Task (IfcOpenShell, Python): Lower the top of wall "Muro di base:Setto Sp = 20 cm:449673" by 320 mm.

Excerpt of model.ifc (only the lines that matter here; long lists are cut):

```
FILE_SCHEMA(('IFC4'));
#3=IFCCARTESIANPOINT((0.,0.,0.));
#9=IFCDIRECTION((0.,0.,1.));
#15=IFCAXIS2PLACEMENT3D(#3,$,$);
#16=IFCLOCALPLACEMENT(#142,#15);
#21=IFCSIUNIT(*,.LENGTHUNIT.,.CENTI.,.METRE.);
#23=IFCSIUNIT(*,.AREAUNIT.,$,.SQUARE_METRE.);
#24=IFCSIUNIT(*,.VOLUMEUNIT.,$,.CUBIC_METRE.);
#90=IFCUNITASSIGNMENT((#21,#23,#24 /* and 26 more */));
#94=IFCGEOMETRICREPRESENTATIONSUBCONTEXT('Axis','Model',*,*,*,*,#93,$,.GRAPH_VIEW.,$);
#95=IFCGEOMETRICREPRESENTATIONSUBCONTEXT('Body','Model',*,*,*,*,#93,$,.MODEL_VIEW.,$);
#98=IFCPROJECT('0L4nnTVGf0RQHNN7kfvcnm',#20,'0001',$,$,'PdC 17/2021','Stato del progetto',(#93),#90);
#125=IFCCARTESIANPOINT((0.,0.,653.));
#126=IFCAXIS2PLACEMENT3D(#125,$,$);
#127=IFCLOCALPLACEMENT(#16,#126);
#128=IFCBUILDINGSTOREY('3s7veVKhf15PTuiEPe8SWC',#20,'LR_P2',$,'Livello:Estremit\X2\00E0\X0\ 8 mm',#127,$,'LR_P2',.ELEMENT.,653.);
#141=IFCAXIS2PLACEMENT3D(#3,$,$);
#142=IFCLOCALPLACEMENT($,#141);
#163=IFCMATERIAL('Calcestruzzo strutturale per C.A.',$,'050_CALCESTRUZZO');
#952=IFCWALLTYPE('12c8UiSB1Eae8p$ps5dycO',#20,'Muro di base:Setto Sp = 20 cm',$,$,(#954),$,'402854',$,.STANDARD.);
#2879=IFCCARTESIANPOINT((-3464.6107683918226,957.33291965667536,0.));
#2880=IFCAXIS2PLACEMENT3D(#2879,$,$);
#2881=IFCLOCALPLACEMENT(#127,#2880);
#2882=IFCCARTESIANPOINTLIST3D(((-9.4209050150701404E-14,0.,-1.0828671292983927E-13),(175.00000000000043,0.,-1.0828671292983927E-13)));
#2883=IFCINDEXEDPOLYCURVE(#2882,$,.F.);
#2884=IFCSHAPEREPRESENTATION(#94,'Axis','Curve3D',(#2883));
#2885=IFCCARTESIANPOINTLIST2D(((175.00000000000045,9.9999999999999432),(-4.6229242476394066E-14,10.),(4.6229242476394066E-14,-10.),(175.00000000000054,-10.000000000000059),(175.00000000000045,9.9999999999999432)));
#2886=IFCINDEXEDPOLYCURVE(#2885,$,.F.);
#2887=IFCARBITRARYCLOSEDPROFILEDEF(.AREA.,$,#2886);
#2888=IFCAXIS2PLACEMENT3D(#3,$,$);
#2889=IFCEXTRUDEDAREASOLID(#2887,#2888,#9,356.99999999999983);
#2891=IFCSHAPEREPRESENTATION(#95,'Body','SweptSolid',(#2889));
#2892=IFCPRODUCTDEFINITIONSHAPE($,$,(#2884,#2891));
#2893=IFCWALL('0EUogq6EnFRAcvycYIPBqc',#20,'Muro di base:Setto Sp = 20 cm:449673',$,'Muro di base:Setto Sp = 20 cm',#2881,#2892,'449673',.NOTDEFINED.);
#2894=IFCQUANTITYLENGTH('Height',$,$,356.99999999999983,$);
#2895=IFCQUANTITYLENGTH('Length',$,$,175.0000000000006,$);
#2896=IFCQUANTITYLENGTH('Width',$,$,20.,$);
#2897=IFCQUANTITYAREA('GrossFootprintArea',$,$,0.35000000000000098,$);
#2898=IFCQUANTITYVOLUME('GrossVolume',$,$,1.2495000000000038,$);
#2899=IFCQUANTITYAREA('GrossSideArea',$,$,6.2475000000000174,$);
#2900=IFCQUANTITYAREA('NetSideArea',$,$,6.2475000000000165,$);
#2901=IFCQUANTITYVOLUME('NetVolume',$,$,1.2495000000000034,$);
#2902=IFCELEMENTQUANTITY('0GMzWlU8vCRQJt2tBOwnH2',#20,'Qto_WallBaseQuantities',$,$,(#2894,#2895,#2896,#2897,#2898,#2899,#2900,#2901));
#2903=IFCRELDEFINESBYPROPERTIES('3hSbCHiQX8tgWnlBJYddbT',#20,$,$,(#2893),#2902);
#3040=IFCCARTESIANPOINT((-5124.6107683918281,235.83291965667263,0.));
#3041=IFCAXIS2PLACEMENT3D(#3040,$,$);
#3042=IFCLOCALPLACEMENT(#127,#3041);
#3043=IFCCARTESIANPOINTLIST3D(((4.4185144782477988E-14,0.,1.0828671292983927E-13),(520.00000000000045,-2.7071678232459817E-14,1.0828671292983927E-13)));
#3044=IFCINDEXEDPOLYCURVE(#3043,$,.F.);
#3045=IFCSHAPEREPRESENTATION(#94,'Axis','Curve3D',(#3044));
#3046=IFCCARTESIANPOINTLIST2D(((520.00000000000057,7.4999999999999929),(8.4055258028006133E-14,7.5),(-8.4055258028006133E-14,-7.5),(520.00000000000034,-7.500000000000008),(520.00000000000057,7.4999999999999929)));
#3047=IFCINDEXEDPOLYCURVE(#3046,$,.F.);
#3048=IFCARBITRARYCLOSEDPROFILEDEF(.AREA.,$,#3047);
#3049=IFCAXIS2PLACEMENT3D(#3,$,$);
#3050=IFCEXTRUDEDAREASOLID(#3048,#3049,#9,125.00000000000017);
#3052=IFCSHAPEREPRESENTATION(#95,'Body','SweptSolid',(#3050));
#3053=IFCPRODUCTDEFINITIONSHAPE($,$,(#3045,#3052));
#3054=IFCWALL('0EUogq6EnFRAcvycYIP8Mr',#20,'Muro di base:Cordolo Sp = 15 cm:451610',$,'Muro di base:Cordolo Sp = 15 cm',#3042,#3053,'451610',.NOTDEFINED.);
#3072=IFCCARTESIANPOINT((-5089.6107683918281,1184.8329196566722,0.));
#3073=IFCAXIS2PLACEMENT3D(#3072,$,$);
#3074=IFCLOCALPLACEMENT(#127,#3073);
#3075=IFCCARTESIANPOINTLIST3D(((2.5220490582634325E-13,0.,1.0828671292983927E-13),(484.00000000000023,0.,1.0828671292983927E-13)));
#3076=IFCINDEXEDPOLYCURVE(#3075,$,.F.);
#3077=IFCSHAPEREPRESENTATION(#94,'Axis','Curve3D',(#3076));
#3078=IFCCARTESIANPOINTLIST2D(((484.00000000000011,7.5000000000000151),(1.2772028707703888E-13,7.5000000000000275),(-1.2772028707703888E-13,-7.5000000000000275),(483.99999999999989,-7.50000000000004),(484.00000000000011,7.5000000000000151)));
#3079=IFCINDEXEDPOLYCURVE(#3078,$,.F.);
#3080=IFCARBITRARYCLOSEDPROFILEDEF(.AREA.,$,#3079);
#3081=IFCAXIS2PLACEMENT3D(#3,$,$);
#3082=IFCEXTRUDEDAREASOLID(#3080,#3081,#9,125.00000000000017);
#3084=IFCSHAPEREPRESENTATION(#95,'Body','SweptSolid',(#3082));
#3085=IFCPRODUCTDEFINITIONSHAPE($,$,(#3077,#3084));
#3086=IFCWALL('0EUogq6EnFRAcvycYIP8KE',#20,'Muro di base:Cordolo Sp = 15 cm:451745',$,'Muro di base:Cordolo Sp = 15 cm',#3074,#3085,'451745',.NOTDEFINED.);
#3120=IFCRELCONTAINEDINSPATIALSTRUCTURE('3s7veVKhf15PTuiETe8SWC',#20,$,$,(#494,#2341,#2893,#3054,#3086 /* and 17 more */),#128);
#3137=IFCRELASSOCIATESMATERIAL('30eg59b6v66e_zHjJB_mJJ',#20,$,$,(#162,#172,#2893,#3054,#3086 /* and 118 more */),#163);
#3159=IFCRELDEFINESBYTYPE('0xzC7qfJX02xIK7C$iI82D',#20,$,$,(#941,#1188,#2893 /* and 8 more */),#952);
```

```python
import ifcopenshell
import ifcopenshell.api.pset
import ifcopenshell.geom
import ifcopenshell.util.element
import ifcopenshell.util.representation
import ifcopenshell.util.shape
import ifcopenshell.util.unit

model = ifcopenshell.open("model.ifc")
unit_scale = ifcopenshell.util.unit.calculate_unit_scale(model)
area_scale = ifcopenshell.util.unit.calculate_unit_scale(model, "AREAUNIT")
volume_scale = ifcopenshell.util.unit.calculate_unit_scale(model, "VOLUMEUNIT")
settings = ifcopenshell.geom.settings()


def volume(element):
    """Net volume in cubic metres, openings subtracted."""
    shape = ifcopenshell.geom.create_shape(settings, element)
    return ifcopenshell.util.shape.get_volume(shape.geometry)


wall = model.by_guid("0EUogq6EnFRAcvycYIPBqc")
before = volume(wall)

body = ifcopenshell.util.representation.get_representation(wall, "Model", "Body")
solid = body.Items[0]
old_height = solid.Depth
solid.Depth -= 0.32 / unit_scale
after = volume(wall)
thickness = 0.2  # wall thickness in metres

# Update the stored height, areas and volumes.
qto = model.by_id(ifcopenshell.util.element.get_pset(wall, "Qto_WallBaseQuantities", should_inherit=False)["id"])
ifcopenshell.api.pset.edit_qto(model, qto=qto, properties={
    "Height": solid.Depth,
    "GrossVolume": ifcopenshell.util.element.get_pset(wall, "Qto_WallBaseQuantities", "GrossVolume") * solid.Depth / old_height,
    "GrossSideArea": ifcopenshell.util.element.get_pset(wall, "Qto_WallBaseQuantities", "GrossSideArea") * solid.Depth / old_height,
    "NetSideArea": after / thickness / area_scale,
    "NetVolume": after / volume_scale,
})

print(f"height {old_height:g} -> {solid.Depth:g}, volume {before:.3f} -> {after:.3f} m3")

model.write("model_edited.ifc")
```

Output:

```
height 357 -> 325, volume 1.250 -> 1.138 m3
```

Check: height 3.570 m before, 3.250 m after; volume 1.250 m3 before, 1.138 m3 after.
